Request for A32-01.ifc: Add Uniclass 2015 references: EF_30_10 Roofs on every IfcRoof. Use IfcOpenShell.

First a look at what the model holds.

```python
import ifcopenshell

model = ifcopenshell.open("A32-01.ifc")
print(model.schema)
print("classifications:", [c.Name for c in model.by_type("IfcClassification")])
for ifc_class in ("IfcDoor", "IfcRoof", "IfcStair", "IfcWall", "IfcWindow"):
    print(ifc_class, len(model.by_type(ifc_class)))
```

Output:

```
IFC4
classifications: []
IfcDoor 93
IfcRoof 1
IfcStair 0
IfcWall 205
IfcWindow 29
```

```python
import ifcopenshell
import ifcopenshell.api.classification

model = ifcopenshell.open("A32-01.ifc")

system = ifcopenshell.api.classification.add_classification(model, classification="Uniclass 2015")

codes = {
    "IfcRoof": ("EF_30_10", "Roofs"),
}
for ifc_class, (code, name) in codes.items():
    products = model.by_type(ifc_class)
    ifcopenshell.api.classification.add_reference(
        model, products=products, classification=system, identification=code, name=name
    )
    print(code, len(products))

model.write("A32-01_rev.ifc")
```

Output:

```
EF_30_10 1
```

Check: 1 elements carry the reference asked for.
